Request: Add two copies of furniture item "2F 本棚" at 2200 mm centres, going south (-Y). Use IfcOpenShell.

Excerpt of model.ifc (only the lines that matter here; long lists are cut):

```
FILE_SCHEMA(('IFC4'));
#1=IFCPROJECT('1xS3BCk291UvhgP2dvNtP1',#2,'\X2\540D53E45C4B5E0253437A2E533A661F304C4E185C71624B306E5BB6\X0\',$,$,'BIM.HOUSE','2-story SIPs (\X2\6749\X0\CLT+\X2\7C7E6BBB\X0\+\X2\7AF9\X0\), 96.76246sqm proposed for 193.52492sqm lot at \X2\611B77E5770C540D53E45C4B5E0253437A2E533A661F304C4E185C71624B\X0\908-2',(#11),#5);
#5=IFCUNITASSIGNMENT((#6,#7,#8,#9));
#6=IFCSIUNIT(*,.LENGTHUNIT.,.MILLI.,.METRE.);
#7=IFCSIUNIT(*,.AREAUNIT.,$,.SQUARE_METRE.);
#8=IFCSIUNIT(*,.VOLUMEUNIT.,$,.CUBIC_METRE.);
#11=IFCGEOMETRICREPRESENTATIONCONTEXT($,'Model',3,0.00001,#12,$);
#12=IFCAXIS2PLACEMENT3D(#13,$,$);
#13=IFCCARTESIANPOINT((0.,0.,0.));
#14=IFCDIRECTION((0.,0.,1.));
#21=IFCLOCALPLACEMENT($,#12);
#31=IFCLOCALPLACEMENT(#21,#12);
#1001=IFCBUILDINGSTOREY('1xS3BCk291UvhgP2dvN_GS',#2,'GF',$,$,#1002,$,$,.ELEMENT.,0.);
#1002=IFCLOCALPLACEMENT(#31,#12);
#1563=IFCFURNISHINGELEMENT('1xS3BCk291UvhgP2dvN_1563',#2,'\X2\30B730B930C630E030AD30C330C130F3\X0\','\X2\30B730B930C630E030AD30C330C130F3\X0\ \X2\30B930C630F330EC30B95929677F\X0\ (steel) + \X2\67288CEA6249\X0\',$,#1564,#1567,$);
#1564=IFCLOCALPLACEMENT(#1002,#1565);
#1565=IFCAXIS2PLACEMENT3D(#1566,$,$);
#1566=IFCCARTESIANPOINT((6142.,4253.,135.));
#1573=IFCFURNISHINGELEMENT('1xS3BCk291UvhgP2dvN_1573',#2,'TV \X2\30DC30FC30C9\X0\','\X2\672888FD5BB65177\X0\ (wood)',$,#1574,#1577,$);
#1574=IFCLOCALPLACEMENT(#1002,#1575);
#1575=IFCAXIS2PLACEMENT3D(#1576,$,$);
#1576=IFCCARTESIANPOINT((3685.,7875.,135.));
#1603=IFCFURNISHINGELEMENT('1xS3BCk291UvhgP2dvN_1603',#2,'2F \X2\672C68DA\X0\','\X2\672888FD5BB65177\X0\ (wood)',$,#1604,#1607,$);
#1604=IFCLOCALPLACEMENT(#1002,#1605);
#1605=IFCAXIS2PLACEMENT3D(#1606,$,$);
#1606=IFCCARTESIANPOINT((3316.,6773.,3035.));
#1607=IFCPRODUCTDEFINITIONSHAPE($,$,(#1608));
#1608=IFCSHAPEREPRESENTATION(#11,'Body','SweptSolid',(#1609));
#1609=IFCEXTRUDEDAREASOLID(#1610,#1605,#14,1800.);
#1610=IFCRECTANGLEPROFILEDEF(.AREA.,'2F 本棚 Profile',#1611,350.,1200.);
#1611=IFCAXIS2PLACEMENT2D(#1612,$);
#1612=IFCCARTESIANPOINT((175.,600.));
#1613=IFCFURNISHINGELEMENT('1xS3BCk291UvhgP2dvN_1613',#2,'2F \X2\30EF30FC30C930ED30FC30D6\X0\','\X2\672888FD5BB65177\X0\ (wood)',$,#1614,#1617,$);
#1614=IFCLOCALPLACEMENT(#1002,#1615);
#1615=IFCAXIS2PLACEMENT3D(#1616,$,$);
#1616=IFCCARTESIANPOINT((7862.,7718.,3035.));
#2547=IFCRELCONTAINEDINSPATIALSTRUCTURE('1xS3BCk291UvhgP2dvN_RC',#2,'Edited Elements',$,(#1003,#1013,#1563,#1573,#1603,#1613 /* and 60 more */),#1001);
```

```python
import numpy as np
import ifcopenshell
import ifcopenshell.api.geometry
import ifcopenshell.api.root
import ifcopenshell.util.element
import ifcopenshell.util.placement
import ifcopenshell.util.unit

model = ifcopenshell.open("model.ifc")
unit_scale = ifcopenshell.util.unit.calculate_unit_scale(model)


def reuse_history(source, copy):
    """copy_class also copies each property set's owner history, people and application; keep the originals."""
    for rel in copy.IsDefinedBy:
        if rel.is_a("IfcRelDefinesByProperties") and (history := rel.RelatingPropertyDefinition.OwnerHistory):
            rel.RelatingPropertyDefinition.OwnerHistory = source.OwnerHistory
            ifcopenshell.util.element.remove_deep2(model, history)


source = model.by_guid("1xS3BCk291UvhgP2dvN_1603")
base = ifcopenshell.util.placement.get_local_placement(source.ObjectPlacement)
step = np.array([0.0, -1.0, 0.0]) * 2.2 / unit_scale

for i in range(1, 3):
    copy = ifcopenshell.api.root.copy_class(model, product=source)
    copy.Representation = ifcopenshell.util.element.copy_deep(
        model, source.Representation, exclude=["IfcGeometricRepresentationContext", "IfcRepresentationMap"]
    )
    reuse_history(source, copy)
    matrix = base.copy()
    matrix[:3, 3] += i * step
    print("added at", matrix[:3, 3].round(3) + 0.0)
    ifcopenshell.api.geometry.edit_object_placement(model, product=copy, matrix=matrix, is_si=False)

model.write("model_updated.ifc")
```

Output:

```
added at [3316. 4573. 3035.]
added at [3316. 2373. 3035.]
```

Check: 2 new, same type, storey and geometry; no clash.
